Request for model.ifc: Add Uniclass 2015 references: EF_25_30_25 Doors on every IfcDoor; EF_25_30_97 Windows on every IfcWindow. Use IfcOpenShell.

First a look at what the model holds.

```python
import ifcopenshell

model = ifcopenshell.open("model.ifc")
print(model.schema)
print("classifications:", [c.Name for c in model.by_type("IfcClassification")])
for ifc_class in ("IfcDoor", "IfcRoof", "IfcStair", "IfcWall", "IfcWindow"):
    print(ifc_class, len(model.by_type(ifc_class)))
```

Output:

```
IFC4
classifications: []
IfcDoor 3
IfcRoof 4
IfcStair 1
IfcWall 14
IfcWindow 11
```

```python
import ifcopenshell
import ifcopenshell.api.classification

model = ifcopenshell.open("model.ifc")

system = ifcopenshell.api.classification.add_classification(model, classification="Uniclass 2015")

codes = {
    "IfcDoor": ("EF_25_30_25", "Doors"),
    "IfcWindow": ("EF_25_30_97", "Windows"),
}
for ifc_class, (code, name) in codes.items():
    products = model.by_type(ifc_class)
    ifcopenshell.api.classification.add_reference(
        model, products=products, classification=system, identification=code, name=name
    )
    print(code, len(products))

model.write("model_v2.ifc")
```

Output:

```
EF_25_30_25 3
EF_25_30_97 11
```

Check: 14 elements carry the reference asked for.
